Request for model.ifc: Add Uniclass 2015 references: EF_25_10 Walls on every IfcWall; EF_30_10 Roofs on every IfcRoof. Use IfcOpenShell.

First a look at what the model holds.

```python
import ifcopenshell

model = ifcopenshell.open("model.ifc")
print(model.schema)
print("classifications:", [c.Name for c in model.by_type("IfcClassification")])
for ifc_class in ("IfcDoor", "IfcRoof", "IfcStair", "IfcWall", "IfcWindow"):
    print(ifc_class, len(model.by_type(ifc_class)))
```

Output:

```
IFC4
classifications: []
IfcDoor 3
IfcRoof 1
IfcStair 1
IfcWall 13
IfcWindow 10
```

```python
import ifcopenshell
import ifcopenshell.api.classification

model = ifcopenshell.open("model.ifc")

system = ifcopenshell.api.classification.add_classification(model, classification="Uniclass 2015")

codes = {
    "IfcWall": ("EF_25_10", "Walls"),
    "IfcRoof": ("EF_30_10", "Roofs"),
}
for ifc_class, (code, name) in codes.items():
    products = model.by_type(ifc_class)
    ifcopenshell.api.classification.add_reference(
        model, products=products, classification=system, identification=code, name=name
    )
    print(code, len(products))

model.write("model_v2.ifc")
```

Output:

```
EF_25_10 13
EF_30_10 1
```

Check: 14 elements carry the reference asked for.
